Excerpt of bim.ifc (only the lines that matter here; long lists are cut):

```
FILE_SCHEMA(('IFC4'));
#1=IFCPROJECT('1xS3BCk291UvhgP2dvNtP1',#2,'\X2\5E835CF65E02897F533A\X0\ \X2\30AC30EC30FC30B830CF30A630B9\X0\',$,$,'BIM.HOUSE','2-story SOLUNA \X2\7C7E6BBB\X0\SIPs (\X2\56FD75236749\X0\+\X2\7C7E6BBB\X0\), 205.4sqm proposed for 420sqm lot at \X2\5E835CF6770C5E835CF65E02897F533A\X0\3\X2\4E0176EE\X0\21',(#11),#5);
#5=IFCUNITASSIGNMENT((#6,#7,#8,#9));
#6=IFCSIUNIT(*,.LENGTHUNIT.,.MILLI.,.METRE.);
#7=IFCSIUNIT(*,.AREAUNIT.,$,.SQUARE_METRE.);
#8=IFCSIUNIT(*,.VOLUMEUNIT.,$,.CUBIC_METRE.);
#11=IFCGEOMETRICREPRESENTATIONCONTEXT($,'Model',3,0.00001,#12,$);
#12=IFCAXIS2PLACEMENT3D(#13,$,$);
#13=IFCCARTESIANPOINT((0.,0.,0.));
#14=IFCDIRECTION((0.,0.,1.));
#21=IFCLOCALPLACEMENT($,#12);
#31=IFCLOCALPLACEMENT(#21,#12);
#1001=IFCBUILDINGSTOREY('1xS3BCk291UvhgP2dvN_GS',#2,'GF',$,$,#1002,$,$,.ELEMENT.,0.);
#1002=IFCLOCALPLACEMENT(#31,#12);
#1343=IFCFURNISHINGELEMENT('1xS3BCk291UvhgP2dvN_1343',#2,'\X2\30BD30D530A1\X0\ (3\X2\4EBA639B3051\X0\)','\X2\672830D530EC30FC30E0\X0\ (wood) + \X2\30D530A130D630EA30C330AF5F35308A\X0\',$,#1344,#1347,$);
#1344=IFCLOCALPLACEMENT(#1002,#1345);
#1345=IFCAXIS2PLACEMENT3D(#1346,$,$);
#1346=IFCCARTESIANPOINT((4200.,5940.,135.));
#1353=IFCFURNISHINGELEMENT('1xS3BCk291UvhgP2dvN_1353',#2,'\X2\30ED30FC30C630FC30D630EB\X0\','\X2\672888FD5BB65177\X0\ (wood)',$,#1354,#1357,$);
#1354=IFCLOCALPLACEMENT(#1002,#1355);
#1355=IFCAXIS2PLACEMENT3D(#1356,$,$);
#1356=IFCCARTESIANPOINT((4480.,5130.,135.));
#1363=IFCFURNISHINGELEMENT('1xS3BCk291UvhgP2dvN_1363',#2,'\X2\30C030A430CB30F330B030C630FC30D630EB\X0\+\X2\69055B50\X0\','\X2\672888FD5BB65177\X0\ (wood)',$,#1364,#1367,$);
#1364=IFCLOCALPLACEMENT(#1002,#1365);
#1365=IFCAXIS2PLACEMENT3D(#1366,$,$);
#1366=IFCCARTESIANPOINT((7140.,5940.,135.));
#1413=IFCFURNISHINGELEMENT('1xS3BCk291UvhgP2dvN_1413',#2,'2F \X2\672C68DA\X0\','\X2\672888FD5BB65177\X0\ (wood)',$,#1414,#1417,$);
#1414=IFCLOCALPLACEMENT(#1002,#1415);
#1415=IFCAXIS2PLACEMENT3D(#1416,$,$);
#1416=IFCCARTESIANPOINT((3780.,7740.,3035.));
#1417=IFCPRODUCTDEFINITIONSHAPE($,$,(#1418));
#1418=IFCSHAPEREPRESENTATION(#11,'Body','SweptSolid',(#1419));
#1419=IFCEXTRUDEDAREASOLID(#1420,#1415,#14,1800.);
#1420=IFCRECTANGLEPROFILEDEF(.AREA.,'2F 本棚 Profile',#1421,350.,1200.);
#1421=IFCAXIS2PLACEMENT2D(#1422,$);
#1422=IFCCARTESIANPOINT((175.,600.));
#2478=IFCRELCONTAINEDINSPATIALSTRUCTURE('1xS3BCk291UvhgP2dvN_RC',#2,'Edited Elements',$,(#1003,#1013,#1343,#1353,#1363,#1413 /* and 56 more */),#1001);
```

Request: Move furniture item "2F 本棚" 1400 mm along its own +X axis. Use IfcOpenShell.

```python
import ifcopenshell
import ifcopenshell.api.geometry
import ifcopenshell.util.placement

model = ifcopenshell.open("bim.ifc")

item = model.by_guid("1xS3BCk291UvhgP2dvN_1413")
matrix = ifcopenshell.util.placement.get_local_placement(item.ObjectPlacement)
matrix[:3, 3] += matrix[:3, 0] * 1400.0
ifcopenshell.api.geometry.edit_object_placement(model, product=item, matrix=matrix, is_si=False)

print(ifcopenshell.util.placement.get_local_placement(item.ObjectPlacement).round(3) + 0.0)

model.write("bim_updated.ifc")
```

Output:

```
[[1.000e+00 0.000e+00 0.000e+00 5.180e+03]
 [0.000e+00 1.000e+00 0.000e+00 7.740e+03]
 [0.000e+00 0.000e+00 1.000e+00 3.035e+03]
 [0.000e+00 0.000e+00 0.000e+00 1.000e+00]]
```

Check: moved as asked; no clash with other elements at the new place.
